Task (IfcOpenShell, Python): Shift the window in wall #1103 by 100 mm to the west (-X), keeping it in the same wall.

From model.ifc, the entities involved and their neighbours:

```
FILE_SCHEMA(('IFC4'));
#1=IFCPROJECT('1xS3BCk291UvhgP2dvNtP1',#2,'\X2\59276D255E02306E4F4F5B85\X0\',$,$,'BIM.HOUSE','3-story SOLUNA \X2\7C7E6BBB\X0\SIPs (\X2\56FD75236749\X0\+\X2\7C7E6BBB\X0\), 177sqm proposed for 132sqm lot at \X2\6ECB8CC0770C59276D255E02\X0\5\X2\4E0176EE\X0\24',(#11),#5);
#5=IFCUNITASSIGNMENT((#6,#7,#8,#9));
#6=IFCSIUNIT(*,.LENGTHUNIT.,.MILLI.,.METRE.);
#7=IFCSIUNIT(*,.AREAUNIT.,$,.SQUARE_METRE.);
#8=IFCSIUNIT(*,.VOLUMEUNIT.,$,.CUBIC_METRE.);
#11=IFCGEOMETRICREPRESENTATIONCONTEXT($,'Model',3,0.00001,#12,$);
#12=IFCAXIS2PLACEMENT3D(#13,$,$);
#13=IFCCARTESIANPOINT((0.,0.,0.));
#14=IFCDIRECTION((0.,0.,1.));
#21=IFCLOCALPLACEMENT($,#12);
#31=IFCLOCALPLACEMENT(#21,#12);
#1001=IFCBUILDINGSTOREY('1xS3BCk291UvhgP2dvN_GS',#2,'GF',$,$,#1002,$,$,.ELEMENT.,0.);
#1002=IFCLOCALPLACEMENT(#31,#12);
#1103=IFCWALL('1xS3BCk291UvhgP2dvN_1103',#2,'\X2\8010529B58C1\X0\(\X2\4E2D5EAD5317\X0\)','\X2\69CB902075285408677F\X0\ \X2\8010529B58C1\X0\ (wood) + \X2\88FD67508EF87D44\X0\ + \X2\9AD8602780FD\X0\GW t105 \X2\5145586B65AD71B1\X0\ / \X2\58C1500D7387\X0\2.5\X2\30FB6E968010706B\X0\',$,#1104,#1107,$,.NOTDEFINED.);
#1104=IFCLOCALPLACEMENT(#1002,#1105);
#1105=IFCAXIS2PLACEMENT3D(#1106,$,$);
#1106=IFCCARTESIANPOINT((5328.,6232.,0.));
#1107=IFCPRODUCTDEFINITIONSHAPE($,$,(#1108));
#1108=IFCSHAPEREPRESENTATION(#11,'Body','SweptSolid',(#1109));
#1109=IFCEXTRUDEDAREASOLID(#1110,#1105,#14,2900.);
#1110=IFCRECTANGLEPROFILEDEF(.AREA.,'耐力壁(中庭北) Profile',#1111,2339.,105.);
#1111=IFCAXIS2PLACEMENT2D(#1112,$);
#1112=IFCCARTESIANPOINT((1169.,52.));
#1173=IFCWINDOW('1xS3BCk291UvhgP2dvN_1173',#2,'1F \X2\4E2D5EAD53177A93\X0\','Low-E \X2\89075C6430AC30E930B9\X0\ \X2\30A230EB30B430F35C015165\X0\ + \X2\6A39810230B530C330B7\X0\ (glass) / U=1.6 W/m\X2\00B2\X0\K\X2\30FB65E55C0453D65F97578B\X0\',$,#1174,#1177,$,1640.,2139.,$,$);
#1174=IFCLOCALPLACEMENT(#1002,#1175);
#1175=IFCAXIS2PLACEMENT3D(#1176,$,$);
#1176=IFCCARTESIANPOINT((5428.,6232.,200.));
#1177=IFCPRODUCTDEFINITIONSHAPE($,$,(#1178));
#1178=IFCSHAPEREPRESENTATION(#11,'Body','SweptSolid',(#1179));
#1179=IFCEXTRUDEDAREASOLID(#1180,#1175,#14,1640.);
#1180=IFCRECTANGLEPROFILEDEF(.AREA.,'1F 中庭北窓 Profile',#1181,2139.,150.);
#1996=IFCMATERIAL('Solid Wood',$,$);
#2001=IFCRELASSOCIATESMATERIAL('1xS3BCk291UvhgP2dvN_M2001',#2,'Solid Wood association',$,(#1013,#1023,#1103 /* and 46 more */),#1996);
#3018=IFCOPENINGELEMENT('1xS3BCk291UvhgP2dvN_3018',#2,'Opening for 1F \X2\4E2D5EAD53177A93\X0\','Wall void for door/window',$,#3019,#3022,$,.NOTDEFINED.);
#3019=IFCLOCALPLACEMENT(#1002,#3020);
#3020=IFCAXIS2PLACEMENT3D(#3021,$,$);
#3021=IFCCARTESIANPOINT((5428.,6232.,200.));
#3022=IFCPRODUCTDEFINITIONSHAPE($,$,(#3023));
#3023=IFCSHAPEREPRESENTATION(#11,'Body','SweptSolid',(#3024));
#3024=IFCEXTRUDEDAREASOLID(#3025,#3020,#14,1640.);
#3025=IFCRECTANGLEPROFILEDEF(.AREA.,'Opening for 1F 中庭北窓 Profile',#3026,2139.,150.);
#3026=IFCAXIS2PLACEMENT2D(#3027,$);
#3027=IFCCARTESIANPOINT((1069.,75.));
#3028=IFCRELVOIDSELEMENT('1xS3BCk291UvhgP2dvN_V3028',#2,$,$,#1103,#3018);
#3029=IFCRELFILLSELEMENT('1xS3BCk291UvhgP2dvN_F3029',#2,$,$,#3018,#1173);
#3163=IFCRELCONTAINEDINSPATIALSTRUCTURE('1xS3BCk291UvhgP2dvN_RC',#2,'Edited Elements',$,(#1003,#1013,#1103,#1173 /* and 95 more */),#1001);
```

```python
import ifcopenshell
import ifcopenshell.api.geometry
import ifcopenshell.util.placement
import ifcopenshell.util.unit

model = ifcopenshell.open("model.ifc")
unit_scale = ifcopenshell.util.unit.calculate_unit_scale(model)

window = model.by_guid("1xS3BCk291UvhgP2dvN_1173")
opening = window.FillsVoids[0].RelatingOpeningElement
wall = opening.VoidsElements[0].RelatingBuildingElement

wall_matrix = ifcopenshell.util.placement.get_local_placement(wall.ObjectPlacement)
shift = wall_matrix[:3, 0] * -0.1 / unit_scale
before = ifcopenshell.util.placement.get_local_placement(window.ObjectPlacement)[:3, 3].copy()

# The window is not placed relative to its opening, so move both.
for product in (opening, window):
    matrix = ifcopenshell.util.placement.get_local_placement(product.ObjectPlacement)
    matrix[:3, 3] += shift
    ifcopenshell.api.geometry.edit_object_placement(model, product=product, matrix=matrix, is_si=False)

after = ifcopenshell.util.placement.get_local_placement(window.ObjectPlacement)[:3, 3]
print("window moved by", (after - before).round(3) + 0.0)

model.write("model_updated.ifc")
```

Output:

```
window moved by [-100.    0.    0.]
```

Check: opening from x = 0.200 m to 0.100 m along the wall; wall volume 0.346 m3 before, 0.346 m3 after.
